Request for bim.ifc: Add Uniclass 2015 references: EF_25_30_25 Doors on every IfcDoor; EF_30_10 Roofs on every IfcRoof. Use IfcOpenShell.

First a look at what the model holds.

```python
import ifcopenshell

model = ifcopenshell.open("bim.ifc")
print(model.schema)
print("classifications:", [c.Name for c in model.by_type("IfcClassification")])
for ifc_class in ("IfcDoor", "IfcRoof", "IfcStair", "IfcWall", "IfcWindow"):
    print(ifc_class, len(model.by_type(ifc_class)))
```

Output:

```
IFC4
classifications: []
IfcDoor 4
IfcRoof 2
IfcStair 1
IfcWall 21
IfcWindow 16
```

```python
import ifcopenshell
import ifcopenshell.api.classification

model = ifcopenshell.open("bim.ifc")

system = ifcopenshell.api.classification.add_classification(model, classification="Uniclass 2015")

codes = {
    "IfcDoor": ("EF_25_30_25", "Doors"),
    "IfcRoof": ("EF_30_10", "Roofs"),
}
for ifc_class, (code, name) in codes.items():
    products = model.by_type(ifc_class)
    ifcopenshell.api.classification.add_reference(
        model, products=products, classification=system, identification=code, name=name
    )
    print(code, len(products))

model.write("bim_rev.ifc")
```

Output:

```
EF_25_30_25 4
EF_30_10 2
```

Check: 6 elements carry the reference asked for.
